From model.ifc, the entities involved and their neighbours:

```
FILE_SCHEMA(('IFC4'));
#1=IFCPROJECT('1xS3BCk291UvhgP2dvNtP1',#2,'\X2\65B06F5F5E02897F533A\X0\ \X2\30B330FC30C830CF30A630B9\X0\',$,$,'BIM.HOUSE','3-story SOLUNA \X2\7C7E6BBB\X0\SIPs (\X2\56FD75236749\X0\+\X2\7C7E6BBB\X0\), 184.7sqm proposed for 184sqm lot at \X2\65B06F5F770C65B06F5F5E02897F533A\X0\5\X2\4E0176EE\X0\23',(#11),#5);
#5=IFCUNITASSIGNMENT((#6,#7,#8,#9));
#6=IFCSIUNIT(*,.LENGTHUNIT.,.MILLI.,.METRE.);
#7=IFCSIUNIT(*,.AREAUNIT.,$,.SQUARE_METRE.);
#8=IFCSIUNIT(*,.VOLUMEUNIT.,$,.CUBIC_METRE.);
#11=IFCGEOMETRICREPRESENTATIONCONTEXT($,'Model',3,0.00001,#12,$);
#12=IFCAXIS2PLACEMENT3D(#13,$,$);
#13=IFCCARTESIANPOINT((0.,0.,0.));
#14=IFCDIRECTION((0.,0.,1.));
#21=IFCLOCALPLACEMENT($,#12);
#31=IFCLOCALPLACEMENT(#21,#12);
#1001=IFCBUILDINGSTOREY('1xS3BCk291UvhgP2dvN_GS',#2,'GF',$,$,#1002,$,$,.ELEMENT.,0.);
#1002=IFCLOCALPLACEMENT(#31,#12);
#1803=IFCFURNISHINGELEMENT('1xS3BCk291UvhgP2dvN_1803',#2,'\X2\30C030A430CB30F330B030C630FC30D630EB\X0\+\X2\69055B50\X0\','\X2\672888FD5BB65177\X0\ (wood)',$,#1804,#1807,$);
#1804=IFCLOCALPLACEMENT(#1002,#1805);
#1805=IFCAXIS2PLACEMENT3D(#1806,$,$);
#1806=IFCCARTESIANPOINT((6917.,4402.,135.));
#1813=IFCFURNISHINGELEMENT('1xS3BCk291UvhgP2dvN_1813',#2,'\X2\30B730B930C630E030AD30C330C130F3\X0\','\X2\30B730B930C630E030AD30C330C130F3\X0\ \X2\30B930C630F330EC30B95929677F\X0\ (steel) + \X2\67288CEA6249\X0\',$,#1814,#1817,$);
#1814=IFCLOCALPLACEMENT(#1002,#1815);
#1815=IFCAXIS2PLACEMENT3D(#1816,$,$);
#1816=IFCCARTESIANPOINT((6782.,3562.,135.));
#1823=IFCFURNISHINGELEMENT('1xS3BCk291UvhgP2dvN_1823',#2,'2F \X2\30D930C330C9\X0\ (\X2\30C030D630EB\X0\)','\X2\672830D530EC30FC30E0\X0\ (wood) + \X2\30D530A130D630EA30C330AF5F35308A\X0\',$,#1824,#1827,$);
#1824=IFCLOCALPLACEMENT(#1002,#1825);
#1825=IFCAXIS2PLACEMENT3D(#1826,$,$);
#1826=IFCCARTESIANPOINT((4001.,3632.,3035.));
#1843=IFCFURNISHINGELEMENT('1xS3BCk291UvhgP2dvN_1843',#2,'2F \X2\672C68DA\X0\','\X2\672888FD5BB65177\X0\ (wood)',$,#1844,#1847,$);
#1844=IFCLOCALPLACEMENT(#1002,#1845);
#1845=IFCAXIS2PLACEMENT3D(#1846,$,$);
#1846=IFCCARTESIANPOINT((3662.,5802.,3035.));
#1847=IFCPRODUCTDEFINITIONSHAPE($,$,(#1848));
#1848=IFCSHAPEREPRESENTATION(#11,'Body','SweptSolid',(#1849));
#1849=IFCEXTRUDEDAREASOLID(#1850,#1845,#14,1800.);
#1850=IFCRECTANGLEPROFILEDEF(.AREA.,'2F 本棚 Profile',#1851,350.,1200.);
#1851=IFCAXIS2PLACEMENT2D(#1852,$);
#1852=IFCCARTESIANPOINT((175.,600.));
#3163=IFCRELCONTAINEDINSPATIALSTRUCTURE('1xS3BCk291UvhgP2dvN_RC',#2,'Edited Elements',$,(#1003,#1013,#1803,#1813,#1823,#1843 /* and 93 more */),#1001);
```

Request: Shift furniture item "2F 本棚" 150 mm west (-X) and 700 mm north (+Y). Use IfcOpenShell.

```python
import ifcopenshell
import ifcopenshell.api.geometry
import ifcopenshell.util.placement
import ifcopenshell.util.unit

model = ifcopenshell.open("model.ifc")
unit_scale = ifcopenshell.util.unit.calculate_unit_scale(model)

item = model.by_guid("1xS3BCk291UvhgP2dvN_1843")
matrix = ifcopenshell.util.placement.get_local_placement(item.ObjectPlacement)
matrix[0, 3] -= 0.15 / unit_scale
matrix[1, 3] += 0.7 / unit_scale
ifcopenshell.api.geometry.edit_object_placement(model, product=item, matrix=matrix, is_si=False)

print(ifcopenshell.util.placement.get_local_placement(item.ObjectPlacement).round(3) + 0.0)

model.write("model_edited.ifc")
```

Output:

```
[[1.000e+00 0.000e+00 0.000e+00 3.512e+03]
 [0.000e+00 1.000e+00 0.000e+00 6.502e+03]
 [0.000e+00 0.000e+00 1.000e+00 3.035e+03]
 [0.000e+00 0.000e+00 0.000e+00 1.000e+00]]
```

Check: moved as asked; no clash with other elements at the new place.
